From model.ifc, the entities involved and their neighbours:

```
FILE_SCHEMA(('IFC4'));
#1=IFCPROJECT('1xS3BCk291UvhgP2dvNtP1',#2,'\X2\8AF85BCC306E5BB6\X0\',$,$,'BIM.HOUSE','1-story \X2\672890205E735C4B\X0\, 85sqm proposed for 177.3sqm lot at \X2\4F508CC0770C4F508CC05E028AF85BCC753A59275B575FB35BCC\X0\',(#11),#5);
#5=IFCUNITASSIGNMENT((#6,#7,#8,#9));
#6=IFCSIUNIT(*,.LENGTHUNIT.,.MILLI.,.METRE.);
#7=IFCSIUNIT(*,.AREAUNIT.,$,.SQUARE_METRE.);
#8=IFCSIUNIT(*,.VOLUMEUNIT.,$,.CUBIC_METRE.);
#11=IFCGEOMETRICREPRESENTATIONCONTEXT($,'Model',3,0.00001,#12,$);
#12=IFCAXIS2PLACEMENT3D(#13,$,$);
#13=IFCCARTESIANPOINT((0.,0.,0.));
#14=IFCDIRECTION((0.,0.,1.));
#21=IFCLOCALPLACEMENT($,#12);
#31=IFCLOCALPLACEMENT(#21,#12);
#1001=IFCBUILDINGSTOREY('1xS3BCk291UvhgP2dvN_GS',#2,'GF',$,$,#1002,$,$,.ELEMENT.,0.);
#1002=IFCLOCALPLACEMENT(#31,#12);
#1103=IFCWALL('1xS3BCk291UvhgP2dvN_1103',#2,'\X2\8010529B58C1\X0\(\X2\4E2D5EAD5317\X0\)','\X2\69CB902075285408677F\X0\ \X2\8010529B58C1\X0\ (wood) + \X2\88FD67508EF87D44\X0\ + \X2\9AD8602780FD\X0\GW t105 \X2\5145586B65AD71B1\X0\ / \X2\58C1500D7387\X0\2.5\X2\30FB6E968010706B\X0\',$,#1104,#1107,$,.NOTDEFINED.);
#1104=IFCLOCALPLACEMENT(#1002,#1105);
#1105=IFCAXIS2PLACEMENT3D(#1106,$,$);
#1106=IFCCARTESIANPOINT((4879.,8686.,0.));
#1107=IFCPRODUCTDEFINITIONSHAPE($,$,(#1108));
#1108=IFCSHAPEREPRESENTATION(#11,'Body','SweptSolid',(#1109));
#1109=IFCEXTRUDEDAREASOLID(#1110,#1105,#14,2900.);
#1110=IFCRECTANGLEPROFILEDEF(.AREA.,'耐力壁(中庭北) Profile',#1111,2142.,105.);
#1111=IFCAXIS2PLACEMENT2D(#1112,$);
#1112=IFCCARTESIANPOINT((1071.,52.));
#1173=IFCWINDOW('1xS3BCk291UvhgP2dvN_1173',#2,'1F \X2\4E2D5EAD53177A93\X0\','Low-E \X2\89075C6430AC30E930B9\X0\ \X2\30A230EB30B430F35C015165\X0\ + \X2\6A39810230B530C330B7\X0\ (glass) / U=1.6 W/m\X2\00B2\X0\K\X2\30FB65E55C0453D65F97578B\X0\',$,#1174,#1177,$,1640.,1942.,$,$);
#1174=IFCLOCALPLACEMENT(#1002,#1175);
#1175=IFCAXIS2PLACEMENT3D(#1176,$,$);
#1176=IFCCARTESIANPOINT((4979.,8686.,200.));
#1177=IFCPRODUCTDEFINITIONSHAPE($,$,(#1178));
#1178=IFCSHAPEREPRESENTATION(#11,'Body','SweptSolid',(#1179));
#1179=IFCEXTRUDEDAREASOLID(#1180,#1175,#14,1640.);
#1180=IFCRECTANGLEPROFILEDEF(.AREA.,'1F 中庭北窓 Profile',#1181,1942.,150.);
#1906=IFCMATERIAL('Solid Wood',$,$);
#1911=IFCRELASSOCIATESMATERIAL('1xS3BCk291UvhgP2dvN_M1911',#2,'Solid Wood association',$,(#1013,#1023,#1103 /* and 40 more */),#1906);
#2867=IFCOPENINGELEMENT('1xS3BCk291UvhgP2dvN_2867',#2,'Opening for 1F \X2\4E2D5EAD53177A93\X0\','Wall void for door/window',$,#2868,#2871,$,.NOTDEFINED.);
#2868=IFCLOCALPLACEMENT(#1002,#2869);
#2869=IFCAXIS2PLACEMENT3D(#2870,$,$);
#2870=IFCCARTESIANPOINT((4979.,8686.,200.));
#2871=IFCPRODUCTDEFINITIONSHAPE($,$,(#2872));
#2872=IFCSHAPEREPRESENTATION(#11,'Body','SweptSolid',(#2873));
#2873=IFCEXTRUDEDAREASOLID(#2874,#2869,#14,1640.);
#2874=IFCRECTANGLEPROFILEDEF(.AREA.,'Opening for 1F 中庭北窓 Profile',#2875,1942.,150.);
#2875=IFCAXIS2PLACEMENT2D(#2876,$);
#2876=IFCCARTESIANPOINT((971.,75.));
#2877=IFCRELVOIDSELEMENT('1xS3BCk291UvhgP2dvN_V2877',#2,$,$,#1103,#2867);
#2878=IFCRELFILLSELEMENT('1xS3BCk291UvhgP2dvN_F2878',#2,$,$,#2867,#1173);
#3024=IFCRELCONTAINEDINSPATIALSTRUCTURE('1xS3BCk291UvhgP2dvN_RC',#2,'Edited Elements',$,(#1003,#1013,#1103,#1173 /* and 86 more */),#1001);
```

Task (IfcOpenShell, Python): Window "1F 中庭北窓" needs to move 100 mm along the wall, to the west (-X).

```python
import ifcopenshell
import ifcopenshell.api.geometry
import ifcopenshell.util.placement
import ifcopenshell.util.unit

model = ifcopenshell.open("model.ifc")
unit_scale = ifcopenshell.util.unit.calculate_unit_scale(model)

window = model.by_id(1173)
opening = window.FillsVoids[0].RelatingOpeningElement
wall = opening.VoidsElements[0].RelatingBuildingElement

wall_matrix = ifcopenshell.util.placement.get_local_placement(wall.ObjectPlacement)
shift = wall_matrix[:3, 0] * -0.1 / unit_scale
before = ifcopenshell.util.placement.get_local_placement(window.ObjectPlacement)[:3, 3].copy()

# The window is not placed relative to its opening, so move both.
for product in (opening, window):
    matrix = ifcopenshell.util.placement.get_local_placement(product.ObjectPlacement)
    matrix[:3, 3] += shift
    ifcopenshell.api.geometry.edit_object_placement(model, product=product, matrix=matrix, is_si=False)

after = ifcopenshell.util.placement.get_local_placement(window.ObjectPlacement)[:3, 3]
print("window moved by", (after - before).round(3) + 0.0)

model.write("model_edited.ifc")
```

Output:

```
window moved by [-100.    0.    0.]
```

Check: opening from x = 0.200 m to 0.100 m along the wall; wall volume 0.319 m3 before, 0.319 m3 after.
